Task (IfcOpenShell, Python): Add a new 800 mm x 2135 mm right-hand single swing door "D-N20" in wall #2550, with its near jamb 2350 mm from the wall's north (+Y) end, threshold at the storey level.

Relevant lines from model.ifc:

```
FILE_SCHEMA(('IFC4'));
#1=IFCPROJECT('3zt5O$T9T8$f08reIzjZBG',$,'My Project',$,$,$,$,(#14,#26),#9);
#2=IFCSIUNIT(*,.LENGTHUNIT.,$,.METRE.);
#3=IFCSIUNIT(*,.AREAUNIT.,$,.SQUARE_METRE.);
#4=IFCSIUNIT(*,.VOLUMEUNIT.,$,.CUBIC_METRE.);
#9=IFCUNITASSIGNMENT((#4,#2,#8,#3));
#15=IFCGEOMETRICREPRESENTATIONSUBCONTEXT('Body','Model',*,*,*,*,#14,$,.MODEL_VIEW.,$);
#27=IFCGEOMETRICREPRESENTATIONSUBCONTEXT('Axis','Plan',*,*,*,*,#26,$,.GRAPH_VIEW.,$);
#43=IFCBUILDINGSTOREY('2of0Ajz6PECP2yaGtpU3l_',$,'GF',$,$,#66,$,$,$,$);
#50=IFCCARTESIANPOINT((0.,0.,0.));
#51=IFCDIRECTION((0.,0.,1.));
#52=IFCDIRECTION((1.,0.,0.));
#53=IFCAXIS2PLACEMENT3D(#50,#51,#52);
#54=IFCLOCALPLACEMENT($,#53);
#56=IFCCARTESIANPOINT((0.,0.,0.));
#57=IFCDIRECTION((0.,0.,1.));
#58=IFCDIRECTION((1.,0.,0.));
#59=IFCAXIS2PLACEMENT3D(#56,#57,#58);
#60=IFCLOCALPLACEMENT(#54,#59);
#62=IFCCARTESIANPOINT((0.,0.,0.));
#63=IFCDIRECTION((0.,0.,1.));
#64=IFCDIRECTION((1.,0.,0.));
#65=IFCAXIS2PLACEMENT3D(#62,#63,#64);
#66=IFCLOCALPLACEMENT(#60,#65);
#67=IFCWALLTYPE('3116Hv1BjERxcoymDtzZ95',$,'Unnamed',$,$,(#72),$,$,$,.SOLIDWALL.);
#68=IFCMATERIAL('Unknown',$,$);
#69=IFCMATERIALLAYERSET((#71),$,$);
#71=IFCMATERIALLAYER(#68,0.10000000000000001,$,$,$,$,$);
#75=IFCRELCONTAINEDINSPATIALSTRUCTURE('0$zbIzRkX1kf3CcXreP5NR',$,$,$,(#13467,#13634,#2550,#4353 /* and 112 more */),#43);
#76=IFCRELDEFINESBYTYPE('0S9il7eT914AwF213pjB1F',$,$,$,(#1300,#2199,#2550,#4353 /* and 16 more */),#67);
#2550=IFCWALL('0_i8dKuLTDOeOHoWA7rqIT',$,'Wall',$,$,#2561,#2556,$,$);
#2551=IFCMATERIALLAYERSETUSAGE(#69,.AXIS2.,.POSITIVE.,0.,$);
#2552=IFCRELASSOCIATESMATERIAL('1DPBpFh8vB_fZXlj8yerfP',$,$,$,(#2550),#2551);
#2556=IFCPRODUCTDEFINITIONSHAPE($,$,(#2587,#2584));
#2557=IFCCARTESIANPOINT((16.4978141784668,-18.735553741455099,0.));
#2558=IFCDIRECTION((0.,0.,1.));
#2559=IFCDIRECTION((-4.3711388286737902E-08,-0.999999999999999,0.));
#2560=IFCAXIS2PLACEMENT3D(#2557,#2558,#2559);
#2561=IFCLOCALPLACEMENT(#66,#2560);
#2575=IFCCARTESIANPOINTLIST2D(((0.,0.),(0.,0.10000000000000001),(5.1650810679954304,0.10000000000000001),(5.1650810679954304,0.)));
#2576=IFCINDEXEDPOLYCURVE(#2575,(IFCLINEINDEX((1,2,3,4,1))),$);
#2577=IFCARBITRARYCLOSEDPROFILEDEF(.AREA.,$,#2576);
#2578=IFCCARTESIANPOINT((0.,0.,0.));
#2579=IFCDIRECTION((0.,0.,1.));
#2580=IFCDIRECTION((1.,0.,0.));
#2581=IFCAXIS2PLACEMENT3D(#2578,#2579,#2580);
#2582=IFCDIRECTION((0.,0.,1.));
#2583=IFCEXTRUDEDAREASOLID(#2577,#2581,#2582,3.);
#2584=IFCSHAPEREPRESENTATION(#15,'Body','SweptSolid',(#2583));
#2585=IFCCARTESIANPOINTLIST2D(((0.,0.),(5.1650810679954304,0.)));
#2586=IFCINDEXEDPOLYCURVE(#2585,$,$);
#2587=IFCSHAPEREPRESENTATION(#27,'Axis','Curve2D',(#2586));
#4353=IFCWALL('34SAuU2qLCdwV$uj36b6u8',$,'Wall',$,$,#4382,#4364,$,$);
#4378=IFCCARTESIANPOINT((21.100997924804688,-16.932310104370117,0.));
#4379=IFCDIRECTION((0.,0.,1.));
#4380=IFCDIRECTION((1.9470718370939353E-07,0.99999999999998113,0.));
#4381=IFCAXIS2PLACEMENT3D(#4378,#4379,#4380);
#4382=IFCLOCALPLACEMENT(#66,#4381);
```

```python
import numpy as np
import ifcopenshell
import ifcopenshell.api.feature
import ifcopenshell.api.geometry
import ifcopenshell.api.root
import ifcopenshell.api.spatial
import ifcopenshell.geom
import ifcopenshell.util.element
import ifcopenshell.util.placement
import ifcopenshell.util.representation
import ifcopenshell.util.shape
import ifcopenshell.util.unit

model = ifcopenshell.open("model.ifc")
unit_scale = ifcopenshell.util.unit.calculate_unit_scale(model)
settings = ifcopenshell.geom.settings()


def volume(element):
    """Net volume in cubic metres, openings subtracted."""
    shape = ifcopenshell.geom.create_shape(settings, element)
    return ifcopenshell.util.shape.get_volume(shape.geometry)


wall = model.by_guid("0_i8dKuLTDOeOHoWA7rqIT")
storey = ifcopenshell.util.element.get_container(wall, ifc_class="IfcBuildingStorey")
context = ifcopenshell.util.representation.get_context(model, "Model", "Body", "MODEL_VIEW")
before = volume(wall)

width, height, from_end, sill = 0.8, 2.135, 2.35, 0.0  # metres

# The wall runs along its own X axis, and the end named is its -X end.
wall_shape = ifcopenshell.geom.create_shape(settings, wall)
x, y, z = ifcopenshell.util.shape.get_vertices(wall_shape.geometry).T
start = x.min() + from_end
face, thickness = float(y.min()), float(y.max() - y.min())
wall_matrix = ifcopenshell.util.placement.get_local_placement(wall.ObjectPlacement)
level = ifcopenshell.util.placement.get_local_placement(storey.ObjectPlacement)[2, 3]


def in_wall(x, y):
    """Placement at x, y metres in the wall's axes, at sill height."""
    matrix = wall_matrix.copy()
    matrix[:, 3] = wall_matrix @ np.array([x / unit_scale, y / unit_scale, 0.0, 1.0])
    matrix[2, 3] = level + sill / unit_scale
    return matrix


# Opening: a box that overshoots both wall faces by 50 mm.
opening = ifcopenshell.api.root.create_entity(model, ifc_class="IfcOpeningElement", predefined_type="OPENING")
box = ifcopenshell.api.geometry.add_wall_representation(
    model, context=context, length=width, height=height, thickness=thickness + 0.1
)
ifcopenshell.api.geometry.assign_representation(model, product=opening, representation=box)
ifcopenshell.api.geometry.edit_object_placement(model, product=opening, matrix=in_wall(start, face - 0.05), is_si=False)
ifcopenshell.api.feature.add_feature(model, feature=opening, element=wall)

door = ifcopenshell.api.root.create_entity(model, ifc_class="IfcDoor", name="D-N20", predefined_type="DOOR")
door.OverallWidth, door.OverallHeight = width / unit_scale, height / unit_scale
door.OperationType = "SINGLE_SWING_RIGHT"
body = ifcopenshell.api.geometry.add_door_representation(
    model,
    context=context,
    overall_width=door.OverallWidth,
    overall_height=door.OverallHeight,
    operation_type="SINGLE_SWING_RIGHT",
    lining_properties={"LiningDepth": thickness / unit_scale, "ThresholdDepth": thickness / unit_scale},
)
ifcopenshell.api.geometry.assign_representation(model, product=door, representation=body)
ifcopenshell.api.spatial.assign_container(model, products=[door], relating_structure=storey)
ifcopenshell.api.feature.add_filling(model, opening=opening, element=door)

# The lining spans the wall, so the door starts at the wall face.
ifcopenshell.api.geometry.edit_object_placement(model, product=door, matrix=in_wall(start, face), is_si=False)

after = volume(wall)

print(f"wall volume {before:.3f} -> {after:.3f} m3")

model.write("model_updated.ifc")
```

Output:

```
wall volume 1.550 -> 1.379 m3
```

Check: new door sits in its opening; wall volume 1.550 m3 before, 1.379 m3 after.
